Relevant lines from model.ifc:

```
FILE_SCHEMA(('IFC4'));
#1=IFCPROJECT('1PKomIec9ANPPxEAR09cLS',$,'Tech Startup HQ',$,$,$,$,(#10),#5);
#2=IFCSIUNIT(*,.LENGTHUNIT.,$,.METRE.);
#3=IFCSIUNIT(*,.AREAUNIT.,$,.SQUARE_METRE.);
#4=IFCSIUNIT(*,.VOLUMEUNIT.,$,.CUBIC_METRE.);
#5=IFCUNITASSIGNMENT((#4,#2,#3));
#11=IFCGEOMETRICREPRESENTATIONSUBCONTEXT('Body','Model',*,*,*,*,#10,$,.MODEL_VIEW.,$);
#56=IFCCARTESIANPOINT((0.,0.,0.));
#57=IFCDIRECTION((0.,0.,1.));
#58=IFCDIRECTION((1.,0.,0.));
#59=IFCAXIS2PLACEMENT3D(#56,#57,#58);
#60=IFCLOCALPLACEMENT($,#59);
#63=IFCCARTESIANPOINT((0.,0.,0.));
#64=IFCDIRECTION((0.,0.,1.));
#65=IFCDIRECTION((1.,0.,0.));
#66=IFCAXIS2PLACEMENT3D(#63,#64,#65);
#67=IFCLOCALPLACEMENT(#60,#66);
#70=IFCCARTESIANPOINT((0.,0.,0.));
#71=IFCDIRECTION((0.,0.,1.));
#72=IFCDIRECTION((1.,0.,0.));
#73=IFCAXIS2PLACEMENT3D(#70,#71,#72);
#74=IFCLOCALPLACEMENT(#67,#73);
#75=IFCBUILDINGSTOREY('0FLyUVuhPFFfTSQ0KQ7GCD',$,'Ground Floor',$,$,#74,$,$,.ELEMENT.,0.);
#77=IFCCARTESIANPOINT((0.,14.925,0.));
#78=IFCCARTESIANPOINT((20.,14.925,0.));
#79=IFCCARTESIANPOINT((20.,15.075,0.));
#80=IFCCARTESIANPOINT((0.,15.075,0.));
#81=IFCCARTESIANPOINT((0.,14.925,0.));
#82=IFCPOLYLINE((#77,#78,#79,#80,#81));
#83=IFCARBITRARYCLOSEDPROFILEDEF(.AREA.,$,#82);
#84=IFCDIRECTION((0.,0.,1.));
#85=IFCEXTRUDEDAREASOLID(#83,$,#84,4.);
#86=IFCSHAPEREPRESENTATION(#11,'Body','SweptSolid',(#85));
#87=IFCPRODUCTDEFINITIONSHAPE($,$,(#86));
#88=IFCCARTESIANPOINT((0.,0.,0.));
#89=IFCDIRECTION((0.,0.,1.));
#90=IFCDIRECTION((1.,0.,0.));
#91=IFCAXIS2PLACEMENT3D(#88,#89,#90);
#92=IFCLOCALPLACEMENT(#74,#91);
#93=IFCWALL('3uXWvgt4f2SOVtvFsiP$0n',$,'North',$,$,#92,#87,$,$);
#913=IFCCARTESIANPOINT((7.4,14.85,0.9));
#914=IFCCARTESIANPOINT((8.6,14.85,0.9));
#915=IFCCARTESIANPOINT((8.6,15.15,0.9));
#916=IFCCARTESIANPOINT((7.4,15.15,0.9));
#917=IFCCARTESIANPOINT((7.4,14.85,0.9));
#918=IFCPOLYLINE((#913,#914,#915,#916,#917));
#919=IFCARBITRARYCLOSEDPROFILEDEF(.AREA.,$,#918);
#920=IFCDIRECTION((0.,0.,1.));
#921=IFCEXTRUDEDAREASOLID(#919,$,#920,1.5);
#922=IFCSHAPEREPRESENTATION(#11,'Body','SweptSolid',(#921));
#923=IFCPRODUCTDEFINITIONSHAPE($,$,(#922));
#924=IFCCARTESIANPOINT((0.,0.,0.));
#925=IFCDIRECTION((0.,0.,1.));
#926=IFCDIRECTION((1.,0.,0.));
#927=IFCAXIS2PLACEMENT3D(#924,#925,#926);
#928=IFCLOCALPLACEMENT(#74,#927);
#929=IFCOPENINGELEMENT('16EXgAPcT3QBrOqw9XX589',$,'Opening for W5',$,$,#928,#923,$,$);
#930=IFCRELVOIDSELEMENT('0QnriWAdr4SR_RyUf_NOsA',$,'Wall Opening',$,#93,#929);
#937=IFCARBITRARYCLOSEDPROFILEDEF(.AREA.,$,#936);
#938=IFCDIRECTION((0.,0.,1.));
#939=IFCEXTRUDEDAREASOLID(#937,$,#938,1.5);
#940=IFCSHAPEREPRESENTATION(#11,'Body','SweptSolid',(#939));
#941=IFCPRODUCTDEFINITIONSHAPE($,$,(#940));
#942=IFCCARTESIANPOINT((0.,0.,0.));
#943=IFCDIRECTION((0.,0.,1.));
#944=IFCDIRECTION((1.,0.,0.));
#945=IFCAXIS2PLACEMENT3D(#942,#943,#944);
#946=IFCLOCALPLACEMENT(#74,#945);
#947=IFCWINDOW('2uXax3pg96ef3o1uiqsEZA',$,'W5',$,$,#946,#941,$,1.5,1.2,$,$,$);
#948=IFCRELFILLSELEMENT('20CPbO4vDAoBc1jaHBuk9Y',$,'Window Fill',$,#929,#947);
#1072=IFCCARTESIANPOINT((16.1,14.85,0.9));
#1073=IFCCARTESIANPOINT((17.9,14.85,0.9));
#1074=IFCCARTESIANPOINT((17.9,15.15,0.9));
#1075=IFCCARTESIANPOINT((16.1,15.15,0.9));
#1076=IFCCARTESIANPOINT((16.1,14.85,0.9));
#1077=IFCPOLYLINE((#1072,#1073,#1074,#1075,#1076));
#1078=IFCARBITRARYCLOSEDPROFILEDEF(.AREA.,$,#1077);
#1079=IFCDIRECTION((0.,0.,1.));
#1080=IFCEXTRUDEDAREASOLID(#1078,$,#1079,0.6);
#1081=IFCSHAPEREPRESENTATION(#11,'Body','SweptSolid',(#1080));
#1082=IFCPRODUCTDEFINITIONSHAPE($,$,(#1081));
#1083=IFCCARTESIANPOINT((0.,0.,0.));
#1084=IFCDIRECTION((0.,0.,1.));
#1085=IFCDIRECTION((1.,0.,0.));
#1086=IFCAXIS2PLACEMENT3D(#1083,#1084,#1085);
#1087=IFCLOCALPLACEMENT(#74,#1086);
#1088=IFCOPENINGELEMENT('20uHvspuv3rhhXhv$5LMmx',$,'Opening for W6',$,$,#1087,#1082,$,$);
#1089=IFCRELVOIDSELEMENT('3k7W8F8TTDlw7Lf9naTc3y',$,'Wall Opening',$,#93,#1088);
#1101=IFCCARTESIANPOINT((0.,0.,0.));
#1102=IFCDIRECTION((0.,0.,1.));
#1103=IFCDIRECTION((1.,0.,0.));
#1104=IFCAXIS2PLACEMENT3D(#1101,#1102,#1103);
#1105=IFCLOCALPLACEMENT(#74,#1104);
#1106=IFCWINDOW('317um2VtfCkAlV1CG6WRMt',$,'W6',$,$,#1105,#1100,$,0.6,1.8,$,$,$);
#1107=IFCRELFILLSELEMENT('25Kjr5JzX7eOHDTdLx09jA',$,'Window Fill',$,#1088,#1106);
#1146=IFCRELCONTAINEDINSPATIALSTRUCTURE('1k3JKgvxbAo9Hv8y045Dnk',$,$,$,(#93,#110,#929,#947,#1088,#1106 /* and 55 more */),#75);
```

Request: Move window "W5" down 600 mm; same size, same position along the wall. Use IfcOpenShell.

```python
import numpy as np
import ifcopenshell
import ifcopenshell.api.geometry
import ifcopenshell.util.placement
import ifcopenshell.util.unit

model = ifcopenshell.open("model.ifc")
unit_scale = ifcopenshell.util.unit.calculate_unit_scale(model)

window = model.by_guid("2uXax3pg96ef3o1uiqsEZA")
opening = window.FillsVoids[0].RelatingOpeningElement
dz = -0.6

shift = np.array([0.0, 0.0, dz])
# The window is not placed relative to its opening, so move both.
for product in (opening, window):
    matrix = ifcopenshell.util.placement.get_local_placement(product.ObjectPlacement)
    matrix[:3, 3] += shift
    ifcopenshell.api.geometry.edit_object_placement(model, product=product, matrix=matrix, is_si=False)

print(f"moved by {dz * unit_scale:+.3f} m")

model.write("model_v2.ifc")
```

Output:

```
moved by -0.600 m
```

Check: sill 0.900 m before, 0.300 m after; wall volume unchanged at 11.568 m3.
